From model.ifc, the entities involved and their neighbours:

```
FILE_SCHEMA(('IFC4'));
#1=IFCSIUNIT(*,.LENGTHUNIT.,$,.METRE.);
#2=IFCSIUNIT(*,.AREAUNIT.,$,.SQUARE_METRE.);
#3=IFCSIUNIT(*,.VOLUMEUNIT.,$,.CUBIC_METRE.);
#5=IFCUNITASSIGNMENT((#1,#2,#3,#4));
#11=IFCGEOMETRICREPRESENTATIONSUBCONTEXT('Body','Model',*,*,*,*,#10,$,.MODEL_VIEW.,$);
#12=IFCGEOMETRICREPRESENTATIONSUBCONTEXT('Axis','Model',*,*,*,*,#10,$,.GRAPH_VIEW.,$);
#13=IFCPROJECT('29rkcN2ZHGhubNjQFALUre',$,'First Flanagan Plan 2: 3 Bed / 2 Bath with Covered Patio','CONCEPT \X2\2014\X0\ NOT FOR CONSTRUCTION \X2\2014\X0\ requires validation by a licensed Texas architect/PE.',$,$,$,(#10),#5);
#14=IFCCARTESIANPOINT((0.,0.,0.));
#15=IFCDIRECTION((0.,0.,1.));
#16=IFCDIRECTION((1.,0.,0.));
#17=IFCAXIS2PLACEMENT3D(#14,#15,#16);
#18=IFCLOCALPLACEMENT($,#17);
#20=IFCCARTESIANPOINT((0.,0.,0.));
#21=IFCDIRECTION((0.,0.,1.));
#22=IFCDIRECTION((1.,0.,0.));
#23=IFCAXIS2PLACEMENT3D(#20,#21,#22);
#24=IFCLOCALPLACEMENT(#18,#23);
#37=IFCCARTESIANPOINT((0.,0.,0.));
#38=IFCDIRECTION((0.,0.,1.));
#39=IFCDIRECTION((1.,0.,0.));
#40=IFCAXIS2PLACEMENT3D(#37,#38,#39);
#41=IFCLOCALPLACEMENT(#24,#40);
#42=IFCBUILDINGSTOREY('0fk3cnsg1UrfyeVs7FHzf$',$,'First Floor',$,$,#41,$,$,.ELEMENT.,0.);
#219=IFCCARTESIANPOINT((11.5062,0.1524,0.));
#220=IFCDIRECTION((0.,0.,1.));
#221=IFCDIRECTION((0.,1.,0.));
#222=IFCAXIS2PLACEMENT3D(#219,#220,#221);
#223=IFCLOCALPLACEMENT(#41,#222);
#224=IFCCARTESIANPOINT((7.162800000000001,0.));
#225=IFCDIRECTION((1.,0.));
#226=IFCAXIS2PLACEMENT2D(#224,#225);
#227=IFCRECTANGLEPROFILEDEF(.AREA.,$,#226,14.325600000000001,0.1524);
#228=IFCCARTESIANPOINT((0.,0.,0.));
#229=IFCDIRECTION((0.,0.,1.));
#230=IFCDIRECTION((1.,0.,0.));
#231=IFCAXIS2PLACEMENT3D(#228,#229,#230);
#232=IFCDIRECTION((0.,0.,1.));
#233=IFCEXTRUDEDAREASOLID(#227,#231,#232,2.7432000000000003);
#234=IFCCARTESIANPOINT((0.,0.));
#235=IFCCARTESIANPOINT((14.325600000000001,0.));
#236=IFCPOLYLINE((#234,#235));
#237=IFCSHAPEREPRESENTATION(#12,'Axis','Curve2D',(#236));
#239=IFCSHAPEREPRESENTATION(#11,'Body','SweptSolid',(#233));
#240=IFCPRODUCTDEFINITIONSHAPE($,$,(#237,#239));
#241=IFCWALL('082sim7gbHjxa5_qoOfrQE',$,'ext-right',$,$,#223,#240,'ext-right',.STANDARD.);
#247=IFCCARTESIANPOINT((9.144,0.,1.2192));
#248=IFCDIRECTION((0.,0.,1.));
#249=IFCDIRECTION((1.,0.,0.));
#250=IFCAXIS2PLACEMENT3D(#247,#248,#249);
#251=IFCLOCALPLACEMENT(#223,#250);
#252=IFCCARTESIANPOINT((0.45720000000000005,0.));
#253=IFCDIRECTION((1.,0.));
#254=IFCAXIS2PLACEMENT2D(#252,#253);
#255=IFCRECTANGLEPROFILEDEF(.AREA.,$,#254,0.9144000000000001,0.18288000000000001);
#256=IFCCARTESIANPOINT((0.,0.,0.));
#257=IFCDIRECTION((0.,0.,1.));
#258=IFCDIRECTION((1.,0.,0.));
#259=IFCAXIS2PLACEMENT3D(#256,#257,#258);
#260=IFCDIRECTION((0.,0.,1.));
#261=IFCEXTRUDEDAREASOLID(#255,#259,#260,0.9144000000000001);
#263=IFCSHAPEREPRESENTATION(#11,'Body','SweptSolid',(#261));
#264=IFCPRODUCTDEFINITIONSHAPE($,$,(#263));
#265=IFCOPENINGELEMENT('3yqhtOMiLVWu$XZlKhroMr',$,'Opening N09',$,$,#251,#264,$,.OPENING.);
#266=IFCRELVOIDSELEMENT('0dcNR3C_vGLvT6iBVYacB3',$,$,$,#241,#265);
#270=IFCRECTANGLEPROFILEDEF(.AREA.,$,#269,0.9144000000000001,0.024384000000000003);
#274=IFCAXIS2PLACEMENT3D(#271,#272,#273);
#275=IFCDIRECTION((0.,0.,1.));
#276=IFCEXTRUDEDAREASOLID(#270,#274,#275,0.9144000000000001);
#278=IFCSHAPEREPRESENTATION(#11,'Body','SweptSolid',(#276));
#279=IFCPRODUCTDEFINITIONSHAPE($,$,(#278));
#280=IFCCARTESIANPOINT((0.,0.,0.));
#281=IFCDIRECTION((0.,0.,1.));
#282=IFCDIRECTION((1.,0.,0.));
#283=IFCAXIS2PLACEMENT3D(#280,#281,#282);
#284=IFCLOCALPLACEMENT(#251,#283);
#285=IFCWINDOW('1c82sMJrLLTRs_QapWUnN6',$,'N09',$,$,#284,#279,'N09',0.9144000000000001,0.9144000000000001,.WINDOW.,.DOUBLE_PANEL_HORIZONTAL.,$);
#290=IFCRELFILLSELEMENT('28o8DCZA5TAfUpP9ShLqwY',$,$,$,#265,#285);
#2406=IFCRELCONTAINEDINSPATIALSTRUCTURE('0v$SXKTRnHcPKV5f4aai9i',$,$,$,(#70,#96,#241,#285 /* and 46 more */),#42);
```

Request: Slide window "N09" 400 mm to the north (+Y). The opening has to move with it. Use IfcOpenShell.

```python
import ifcopenshell
import ifcopenshell.api.geometry
import ifcopenshell.util.placement
import ifcopenshell.util.unit

model = ifcopenshell.open("model.ifc")
unit_scale = ifcopenshell.util.unit.calculate_unit_scale(model)

window = model.by_id(285)
opening = window.FillsVoids[0].RelatingOpeningElement
wall = opening.VoidsElements[0].RelatingBuildingElement

wall_matrix = ifcopenshell.util.placement.get_local_placement(wall.ObjectPlacement)
shift = wall_matrix[:3, 0] * 0.4 / unit_scale
before = ifcopenshell.util.placement.get_local_placement(window.ObjectPlacement)[:3, 3].copy()

# The window is placed relative to its opening, so it follows when the opening moves.
matrix = ifcopenshell.util.placement.get_local_placement(opening.ObjectPlacement)
matrix[:3, 3] += shift
ifcopenshell.api.geometry.edit_object_placement(
    model, product=opening, matrix=matrix, is_si=False, should_transform_children=True
)

after = ifcopenshell.util.placement.get_local_placement(window.ObjectPlacement)[:3, 3]
print("window moved by", (after - before).round(3) + 0.0)

model.write("model-out.ifc")
```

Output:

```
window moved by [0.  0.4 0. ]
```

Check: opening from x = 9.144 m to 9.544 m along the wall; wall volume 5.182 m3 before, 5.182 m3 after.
